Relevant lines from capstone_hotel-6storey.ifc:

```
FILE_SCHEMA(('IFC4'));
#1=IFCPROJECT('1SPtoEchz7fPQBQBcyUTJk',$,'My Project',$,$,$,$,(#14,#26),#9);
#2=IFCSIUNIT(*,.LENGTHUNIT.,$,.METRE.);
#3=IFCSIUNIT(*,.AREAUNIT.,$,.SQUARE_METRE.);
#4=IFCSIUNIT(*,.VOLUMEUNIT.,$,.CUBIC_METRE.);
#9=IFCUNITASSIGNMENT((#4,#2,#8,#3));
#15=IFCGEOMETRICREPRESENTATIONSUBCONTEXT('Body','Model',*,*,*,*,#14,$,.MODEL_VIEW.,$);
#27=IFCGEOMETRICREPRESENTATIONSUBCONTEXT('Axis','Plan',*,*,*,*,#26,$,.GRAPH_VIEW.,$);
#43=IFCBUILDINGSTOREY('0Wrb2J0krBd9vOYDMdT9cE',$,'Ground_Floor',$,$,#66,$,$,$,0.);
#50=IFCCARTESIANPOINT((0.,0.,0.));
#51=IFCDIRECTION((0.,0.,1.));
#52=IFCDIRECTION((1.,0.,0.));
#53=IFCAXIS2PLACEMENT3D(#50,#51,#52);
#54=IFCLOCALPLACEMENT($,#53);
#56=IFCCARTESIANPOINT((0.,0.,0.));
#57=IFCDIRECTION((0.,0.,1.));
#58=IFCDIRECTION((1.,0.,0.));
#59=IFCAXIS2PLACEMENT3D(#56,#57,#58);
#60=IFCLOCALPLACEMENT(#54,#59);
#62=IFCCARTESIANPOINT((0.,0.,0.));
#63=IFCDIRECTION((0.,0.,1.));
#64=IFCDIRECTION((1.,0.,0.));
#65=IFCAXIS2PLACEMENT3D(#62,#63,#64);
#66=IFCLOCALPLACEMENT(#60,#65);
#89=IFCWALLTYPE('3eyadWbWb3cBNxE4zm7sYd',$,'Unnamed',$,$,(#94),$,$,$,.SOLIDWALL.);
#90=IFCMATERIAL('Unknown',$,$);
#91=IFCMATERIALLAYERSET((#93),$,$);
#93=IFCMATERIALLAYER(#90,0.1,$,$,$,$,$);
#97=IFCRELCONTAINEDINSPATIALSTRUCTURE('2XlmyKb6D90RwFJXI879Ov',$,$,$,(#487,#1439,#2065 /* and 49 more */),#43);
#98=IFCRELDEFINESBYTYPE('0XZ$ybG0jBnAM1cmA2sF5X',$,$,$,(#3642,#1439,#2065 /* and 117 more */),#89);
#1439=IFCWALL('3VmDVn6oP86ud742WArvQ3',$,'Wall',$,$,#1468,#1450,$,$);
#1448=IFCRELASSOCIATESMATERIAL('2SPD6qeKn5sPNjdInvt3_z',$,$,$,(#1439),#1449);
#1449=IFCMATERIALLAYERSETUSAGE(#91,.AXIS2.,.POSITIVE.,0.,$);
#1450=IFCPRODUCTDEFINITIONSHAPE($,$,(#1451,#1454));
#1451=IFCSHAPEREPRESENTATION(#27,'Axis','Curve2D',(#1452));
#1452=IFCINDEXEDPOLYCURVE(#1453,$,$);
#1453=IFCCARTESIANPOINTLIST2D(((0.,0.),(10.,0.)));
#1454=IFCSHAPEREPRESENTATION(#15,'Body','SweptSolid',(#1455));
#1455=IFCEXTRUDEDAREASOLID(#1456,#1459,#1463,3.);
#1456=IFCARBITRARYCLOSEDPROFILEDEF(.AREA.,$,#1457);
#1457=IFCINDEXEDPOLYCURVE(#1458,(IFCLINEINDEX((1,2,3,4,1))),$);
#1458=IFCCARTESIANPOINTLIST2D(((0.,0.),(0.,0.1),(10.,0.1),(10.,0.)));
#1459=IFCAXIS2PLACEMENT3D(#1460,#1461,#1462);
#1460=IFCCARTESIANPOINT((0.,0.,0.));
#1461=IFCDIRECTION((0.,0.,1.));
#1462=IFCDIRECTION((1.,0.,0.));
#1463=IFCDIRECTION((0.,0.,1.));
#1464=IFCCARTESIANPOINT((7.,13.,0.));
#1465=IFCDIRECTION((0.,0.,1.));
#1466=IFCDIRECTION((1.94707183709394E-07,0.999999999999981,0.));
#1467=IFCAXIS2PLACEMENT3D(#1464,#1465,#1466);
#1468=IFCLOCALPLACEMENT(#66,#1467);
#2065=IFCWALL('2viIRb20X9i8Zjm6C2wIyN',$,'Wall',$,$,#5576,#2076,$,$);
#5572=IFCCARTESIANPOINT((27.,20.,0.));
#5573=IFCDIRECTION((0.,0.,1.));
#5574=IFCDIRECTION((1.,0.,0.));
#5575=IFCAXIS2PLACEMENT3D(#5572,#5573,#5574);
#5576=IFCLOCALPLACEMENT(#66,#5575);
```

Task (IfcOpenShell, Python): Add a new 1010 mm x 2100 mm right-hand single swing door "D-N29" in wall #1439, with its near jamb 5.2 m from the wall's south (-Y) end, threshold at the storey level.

```python
import numpy as np
import ifcopenshell
import ifcopenshell.api.feature
import ifcopenshell.api.geometry
import ifcopenshell.api.root
import ifcopenshell.api.spatial
import ifcopenshell.geom
import ifcopenshell.util.element
import ifcopenshell.util.placement
import ifcopenshell.util.representation
import ifcopenshell.util.shape
import ifcopenshell.util.unit

model = ifcopenshell.open("capstone_hotel-6storey.ifc")
unit_scale = ifcopenshell.util.unit.calculate_unit_scale(model)
settings = ifcopenshell.geom.settings()


def volume(element):
    """Net volume in cubic metres, openings subtracted."""
    shape = ifcopenshell.geom.create_shape(settings, element)
    return ifcopenshell.util.shape.get_volume(shape.geometry)


wall = model.by_guid("3VmDVn6oP86ud742WArvQ3")
storey = ifcopenshell.util.element.get_container(wall, ifc_class="IfcBuildingStorey")
context = ifcopenshell.util.representation.get_context(model, "Model", "Body", "MODEL_VIEW")
before = volume(wall)

width, height, from_end, sill = 1.01, 2.1, 5.2, 0.0  # metres

# The wall runs along its own X axis, and the end named is its -X end.
wall_shape = ifcopenshell.geom.create_shape(settings, wall)
x, y, z = ifcopenshell.util.shape.get_vertices(wall_shape.geometry).T
start = x.min() + from_end
face, thickness = float(y.min()), float(y.max() - y.min())
wall_matrix = ifcopenshell.util.placement.get_local_placement(wall.ObjectPlacement)
level = ifcopenshell.util.placement.get_local_placement(storey.ObjectPlacement)[2, 3]


def in_wall(x, y):
    """Placement at x, y metres in the wall's axes, at sill height."""
    matrix = wall_matrix.copy()
    matrix[:, 3] = wall_matrix @ np.array([x / unit_scale, y / unit_scale, 0.0, 1.0])
    matrix[2, 3] = level + sill / unit_scale
    return matrix


# Opening: a box that overshoots both wall faces by 50 mm.
opening = ifcopenshell.api.root.create_entity(model, ifc_class="IfcOpeningElement", predefined_type="OPENING")
box = ifcopenshell.api.geometry.add_wall_representation(
    model, context=context, length=width, height=height, thickness=thickness + 0.1
)
ifcopenshell.api.geometry.assign_representation(model, product=opening, representation=box)
ifcopenshell.api.geometry.edit_object_placement(model, product=opening, matrix=in_wall(start, face - 0.05), is_si=False)
ifcopenshell.api.feature.add_feature(model, feature=opening, element=wall)

door = ifcopenshell.api.root.create_entity(model, ifc_class="IfcDoor", name="D-N29", predefined_type="DOOR")
door.OverallWidth, door.OverallHeight = width / unit_scale, height / unit_scale
door.OperationType = "SINGLE_SWING_RIGHT"
body = ifcopenshell.api.geometry.add_door_representation(
    model,
    context=context,
    overall_width=door.OverallWidth,
    overall_height=door.OverallHeight,
    operation_type="SINGLE_SWING_RIGHT",
    lining_properties={"LiningDepth": thickness / unit_scale, "ThresholdDepth": thickness / unit_scale},
)
ifcopenshell.api.geometry.assign_representation(model, product=door, representation=body)
ifcopenshell.api.spatial.assign_container(model, products=[door], relating_structure=storey)
ifcopenshell.api.feature.add_filling(model, opening=opening, element=door)

# The lining spans the wall, so the door starts at the wall face.
ifcopenshell.api.geometry.edit_object_placement(model, product=door, matrix=in_wall(start, face), is_si=False)

after = volume(wall)

print(f"wall volume {before:.3f} -> {after:.3f} m3")

model.write("capstone_hotel-6storey_edited.ifc")
```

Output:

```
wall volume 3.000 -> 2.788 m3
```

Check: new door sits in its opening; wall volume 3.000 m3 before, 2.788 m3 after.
